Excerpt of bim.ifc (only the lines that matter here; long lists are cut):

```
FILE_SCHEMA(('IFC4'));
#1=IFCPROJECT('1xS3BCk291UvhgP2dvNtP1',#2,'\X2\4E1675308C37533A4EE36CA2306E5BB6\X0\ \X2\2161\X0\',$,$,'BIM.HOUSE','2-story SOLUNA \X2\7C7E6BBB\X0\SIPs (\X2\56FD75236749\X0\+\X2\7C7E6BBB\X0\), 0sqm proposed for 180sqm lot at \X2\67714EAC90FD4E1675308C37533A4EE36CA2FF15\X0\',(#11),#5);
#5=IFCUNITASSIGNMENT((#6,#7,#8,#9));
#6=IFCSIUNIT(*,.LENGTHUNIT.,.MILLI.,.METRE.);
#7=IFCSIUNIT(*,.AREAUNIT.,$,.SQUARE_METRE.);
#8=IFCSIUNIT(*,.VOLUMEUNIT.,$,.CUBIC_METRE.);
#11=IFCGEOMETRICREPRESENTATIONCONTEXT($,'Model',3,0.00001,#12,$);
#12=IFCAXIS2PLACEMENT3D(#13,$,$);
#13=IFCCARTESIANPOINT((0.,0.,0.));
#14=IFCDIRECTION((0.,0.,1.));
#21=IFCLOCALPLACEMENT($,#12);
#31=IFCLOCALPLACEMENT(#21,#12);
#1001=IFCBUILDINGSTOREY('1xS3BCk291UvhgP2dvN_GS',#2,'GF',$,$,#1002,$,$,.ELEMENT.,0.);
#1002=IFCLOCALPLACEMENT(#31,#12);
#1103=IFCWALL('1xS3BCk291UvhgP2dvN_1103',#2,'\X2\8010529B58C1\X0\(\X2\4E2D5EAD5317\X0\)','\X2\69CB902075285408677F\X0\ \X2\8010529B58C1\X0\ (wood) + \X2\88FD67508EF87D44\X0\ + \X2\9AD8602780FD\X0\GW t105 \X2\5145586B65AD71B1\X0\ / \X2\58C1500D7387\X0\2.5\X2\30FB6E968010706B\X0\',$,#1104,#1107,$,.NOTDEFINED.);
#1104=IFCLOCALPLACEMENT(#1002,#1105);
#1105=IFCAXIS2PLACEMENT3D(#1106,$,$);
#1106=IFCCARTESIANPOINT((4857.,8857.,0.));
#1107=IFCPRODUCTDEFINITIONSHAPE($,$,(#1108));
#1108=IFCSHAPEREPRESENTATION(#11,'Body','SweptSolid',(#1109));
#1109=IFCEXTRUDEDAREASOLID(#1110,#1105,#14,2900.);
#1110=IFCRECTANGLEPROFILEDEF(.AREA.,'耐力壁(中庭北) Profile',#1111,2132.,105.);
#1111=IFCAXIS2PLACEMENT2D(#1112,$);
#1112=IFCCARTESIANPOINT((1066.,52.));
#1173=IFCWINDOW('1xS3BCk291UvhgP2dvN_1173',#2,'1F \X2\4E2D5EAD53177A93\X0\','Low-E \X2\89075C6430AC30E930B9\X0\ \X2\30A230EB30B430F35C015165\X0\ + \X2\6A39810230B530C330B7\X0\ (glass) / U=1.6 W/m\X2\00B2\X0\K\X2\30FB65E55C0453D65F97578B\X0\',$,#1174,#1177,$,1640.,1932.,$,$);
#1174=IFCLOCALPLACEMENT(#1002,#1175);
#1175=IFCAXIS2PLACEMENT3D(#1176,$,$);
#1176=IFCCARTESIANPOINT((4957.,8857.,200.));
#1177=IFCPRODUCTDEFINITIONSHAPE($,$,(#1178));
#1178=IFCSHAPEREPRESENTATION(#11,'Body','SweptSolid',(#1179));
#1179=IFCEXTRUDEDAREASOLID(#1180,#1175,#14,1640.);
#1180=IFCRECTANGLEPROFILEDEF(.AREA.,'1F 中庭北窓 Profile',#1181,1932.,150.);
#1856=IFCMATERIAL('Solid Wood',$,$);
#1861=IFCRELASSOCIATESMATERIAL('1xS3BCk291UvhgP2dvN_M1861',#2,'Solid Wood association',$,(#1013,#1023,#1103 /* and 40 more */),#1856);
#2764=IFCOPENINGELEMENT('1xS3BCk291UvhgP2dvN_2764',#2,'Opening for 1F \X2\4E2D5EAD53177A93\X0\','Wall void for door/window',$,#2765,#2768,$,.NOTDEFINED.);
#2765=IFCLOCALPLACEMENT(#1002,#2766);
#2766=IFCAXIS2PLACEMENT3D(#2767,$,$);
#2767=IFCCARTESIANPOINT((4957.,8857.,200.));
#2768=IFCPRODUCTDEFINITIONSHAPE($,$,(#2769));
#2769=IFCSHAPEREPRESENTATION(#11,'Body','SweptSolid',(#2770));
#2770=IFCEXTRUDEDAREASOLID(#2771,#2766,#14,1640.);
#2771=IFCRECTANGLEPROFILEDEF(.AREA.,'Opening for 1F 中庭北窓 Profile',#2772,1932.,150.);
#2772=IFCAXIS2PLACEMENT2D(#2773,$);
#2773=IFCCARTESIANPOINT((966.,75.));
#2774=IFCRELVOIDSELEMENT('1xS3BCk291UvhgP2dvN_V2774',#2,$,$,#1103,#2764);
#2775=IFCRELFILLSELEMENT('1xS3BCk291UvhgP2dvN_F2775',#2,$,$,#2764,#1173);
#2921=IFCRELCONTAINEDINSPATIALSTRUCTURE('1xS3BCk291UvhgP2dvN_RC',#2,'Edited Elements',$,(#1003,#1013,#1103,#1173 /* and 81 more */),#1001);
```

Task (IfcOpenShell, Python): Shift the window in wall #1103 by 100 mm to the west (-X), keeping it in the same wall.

```python
import ifcopenshell
import ifcopenshell.api.geometry
import ifcopenshell.util.placement

model = ifcopenshell.open("bim.ifc")

window = model.by_guid("1xS3BCk291UvhgP2dvN_1173")
opening = window.FillsVoids[0].RelatingOpeningElement
wall = opening.VoidsElements[0].RelatingBuildingElement

wall_matrix = ifcopenshell.util.placement.get_local_placement(wall.ObjectPlacement)
shift = wall_matrix[:3, 0] * -100.0
before = ifcopenshell.util.placement.get_local_placement(window.ObjectPlacement)[:3, 3].copy()

# The window is not placed relative to its opening, so move both.
for product in (opening, window):
    matrix = ifcopenshell.util.placement.get_local_placement(product.ObjectPlacement)
    matrix[:3, 3] += shift
    ifcopenshell.api.geometry.edit_object_placement(model, product=product, matrix=matrix, is_si=False)

after = ifcopenshell.util.placement.get_local_placement(window.ObjectPlacement)[:3, 3]
print("window moved by", (after - before).round(3) + 0.0)

model.write("bim_edited.ifc")
```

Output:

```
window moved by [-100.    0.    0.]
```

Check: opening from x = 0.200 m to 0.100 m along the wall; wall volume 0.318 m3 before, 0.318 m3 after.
